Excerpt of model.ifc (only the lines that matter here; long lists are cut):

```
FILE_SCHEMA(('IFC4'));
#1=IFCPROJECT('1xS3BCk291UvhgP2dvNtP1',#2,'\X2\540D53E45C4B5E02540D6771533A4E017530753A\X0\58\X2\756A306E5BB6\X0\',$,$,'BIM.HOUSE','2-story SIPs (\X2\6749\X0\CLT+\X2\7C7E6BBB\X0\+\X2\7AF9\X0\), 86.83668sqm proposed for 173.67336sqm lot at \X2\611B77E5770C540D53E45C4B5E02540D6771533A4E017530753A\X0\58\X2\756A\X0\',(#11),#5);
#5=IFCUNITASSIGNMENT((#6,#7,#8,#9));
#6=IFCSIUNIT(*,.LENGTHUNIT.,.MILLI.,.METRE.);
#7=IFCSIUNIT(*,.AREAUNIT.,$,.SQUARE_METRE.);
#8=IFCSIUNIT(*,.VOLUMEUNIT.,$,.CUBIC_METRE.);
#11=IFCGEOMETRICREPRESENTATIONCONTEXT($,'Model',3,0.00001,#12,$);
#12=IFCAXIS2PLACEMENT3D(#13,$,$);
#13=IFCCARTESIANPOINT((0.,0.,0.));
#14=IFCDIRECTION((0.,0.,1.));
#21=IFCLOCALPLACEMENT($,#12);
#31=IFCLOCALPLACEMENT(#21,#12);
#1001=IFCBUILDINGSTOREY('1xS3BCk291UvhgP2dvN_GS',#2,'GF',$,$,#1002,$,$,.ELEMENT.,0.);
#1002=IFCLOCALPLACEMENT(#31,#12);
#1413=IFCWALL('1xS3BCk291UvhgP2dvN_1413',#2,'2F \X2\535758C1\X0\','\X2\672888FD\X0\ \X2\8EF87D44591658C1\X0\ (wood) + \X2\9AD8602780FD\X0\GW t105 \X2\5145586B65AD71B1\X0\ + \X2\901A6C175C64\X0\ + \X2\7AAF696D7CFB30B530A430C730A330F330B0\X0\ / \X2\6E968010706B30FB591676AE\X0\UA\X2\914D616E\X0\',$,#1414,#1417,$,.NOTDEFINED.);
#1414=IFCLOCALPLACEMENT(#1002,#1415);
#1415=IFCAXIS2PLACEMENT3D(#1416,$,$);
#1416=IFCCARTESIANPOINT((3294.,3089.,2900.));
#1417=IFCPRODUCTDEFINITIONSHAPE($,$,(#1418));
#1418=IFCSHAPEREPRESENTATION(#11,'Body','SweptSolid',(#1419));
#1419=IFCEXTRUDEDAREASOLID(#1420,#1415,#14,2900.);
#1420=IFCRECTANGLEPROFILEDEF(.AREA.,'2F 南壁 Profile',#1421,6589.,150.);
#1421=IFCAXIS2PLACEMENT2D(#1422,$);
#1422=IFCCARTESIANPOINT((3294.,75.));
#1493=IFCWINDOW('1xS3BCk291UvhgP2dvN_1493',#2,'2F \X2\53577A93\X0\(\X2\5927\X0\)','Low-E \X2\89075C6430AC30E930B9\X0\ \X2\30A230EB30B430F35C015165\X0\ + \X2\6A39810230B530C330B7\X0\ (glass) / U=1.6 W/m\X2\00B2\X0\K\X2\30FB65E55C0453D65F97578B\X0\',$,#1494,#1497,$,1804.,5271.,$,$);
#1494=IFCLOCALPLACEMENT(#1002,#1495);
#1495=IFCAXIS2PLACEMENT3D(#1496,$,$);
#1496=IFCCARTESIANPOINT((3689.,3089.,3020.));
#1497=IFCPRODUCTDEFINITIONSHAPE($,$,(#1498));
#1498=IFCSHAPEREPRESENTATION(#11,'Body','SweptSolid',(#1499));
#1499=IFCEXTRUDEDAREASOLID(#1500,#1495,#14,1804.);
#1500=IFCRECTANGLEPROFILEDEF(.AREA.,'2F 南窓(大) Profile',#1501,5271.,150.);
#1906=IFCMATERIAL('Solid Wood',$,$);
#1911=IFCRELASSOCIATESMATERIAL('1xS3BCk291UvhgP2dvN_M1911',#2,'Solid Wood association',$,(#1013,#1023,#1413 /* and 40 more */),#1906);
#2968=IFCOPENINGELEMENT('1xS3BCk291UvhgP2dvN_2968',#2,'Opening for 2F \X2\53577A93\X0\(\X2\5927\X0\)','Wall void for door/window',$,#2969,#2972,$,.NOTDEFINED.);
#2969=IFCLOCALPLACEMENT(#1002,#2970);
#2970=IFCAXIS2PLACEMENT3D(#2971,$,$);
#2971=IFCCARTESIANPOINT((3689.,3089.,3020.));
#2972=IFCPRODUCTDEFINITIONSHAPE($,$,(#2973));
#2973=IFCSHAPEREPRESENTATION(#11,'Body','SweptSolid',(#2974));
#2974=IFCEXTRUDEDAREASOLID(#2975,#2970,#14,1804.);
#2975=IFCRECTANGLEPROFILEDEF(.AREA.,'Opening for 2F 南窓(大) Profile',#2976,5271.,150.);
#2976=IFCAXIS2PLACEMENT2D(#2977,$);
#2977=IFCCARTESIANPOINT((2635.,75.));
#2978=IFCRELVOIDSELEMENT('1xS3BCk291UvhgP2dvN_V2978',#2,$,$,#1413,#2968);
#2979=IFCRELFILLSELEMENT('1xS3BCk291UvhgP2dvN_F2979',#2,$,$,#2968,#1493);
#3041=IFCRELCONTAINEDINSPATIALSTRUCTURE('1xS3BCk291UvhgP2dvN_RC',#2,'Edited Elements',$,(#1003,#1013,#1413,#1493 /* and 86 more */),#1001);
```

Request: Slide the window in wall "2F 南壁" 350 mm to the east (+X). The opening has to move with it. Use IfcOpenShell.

```python
import ifcopenshell
import ifcopenshell.api.geometry
import ifcopenshell.util.placement
import ifcopenshell.util.unit

model = ifcopenshell.open("model.ifc")
unit_scale = ifcopenshell.util.unit.calculate_unit_scale(model)

window = model.by_guid("1xS3BCk291UvhgP2dvN_1493")
opening = window.FillsVoids[0].RelatingOpeningElement
wall = opening.VoidsElements[0].RelatingBuildingElement

wall_matrix = ifcopenshell.util.placement.get_local_placement(wall.ObjectPlacement)
shift = wall_matrix[:3, 0] * 0.35 / unit_scale
before = ifcopenshell.util.placement.get_local_placement(window.ObjectPlacement)[:3, 3].copy()

# The window is not placed relative to its opening, so move both.
for product in (opening, window):
    matrix = ifcopenshell.util.placement.get_local_placement(product.ObjectPlacement)
    matrix[:3, 3] += shift
    ifcopenshell.api.geometry.edit_object_placement(model, product=product, matrix=matrix, is_si=False)

after = ifcopenshell.util.placement.get_local_placement(window.ObjectPlacement)[:3, 3]
print("window moved by", (after - before).round(3) + 0.0)

model.write("model_v2.ifc")
```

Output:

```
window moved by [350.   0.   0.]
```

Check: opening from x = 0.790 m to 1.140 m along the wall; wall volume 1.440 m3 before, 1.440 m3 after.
